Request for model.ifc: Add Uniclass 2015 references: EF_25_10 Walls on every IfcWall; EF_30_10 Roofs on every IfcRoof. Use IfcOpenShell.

First a look at what the model holds.

```python
import ifcopenshell

model = ifcopenshell.open("model.ifc")
print(model.schema)
print("classifications:", [c.Name for c in model.by_type("IfcClassification")])
for ifc_class in ("IfcDoor", "IfcRoof", "IfcStair", "IfcWall", "IfcWindow"):
    print(ifc_class, len(model.by_type(ifc_class)))
```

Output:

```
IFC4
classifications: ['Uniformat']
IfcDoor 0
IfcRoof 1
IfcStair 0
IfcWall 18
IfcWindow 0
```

```python
import ifcopenshell
import ifcopenshell.api.classification

model = ifcopenshell.open("model.ifc")

system = ifcopenshell.api.classification.add_classification(model, classification="Uniclass 2015")

codes = {
    "IfcWall": ("EF_25_10", "Walls"),
    "IfcRoof": ("EF_30_10", "Roofs"),
}
for ifc_class, (code, name) in codes.items():
    products = model.by_type(ifc_class)
    ifcopenshell.api.classification.add_reference(
        model, products=products, classification=system, identification=code, name=name
    )
    print(code, len(products))

model.write("model_updated.ifc")
```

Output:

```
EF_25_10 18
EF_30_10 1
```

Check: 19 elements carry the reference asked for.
